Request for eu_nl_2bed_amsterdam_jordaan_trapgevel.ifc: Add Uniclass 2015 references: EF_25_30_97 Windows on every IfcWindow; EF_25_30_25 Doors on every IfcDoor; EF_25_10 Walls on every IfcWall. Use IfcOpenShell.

First a look at what the model holds.

```python
import ifcopenshell

model = ifcopenshell.open("eu_nl_2bed_amsterdam_jordaan_trapgevel.ifc")
print(model.schema)
print("classifications:", [c.Name for c in model.by_type("IfcClassification")])
for ifc_class in ("IfcDoor", "IfcRoof", "IfcStair", "IfcWall", "IfcWindow"):
    print(ifc_class, len(model.by_type(ifc_class)))
```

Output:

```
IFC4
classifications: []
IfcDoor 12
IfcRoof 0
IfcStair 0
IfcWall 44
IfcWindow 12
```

```python
import ifcopenshell
import ifcopenshell.api.classification

model = ifcopenshell.open("eu_nl_2bed_amsterdam_jordaan_trapgevel.ifc")

system = ifcopenshell.api.classification.add_classification(model, classification="Uniclass 2015")

codes = {
    "IfcWindow": ("EF_25_30_97", "Windows"),
    "IfcDoor": ("EF_25_30_25", "Doors"),
    "IfcWall": ("EF_25_10", "Walls"),
}
for ifc_class, (code, name) in codes.items():
    products = model.by_type(ifc_class)
    ifcopenshell.api.classification.add_reference(
        model, products=products, classification=system, identification=code, name=name
    )
    print(code, len(products))

model.write("eu_nl_2bed_amsterdam_jordaan_trapgevel-out.ifc")
```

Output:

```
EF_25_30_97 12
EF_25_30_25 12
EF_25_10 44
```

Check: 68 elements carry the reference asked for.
